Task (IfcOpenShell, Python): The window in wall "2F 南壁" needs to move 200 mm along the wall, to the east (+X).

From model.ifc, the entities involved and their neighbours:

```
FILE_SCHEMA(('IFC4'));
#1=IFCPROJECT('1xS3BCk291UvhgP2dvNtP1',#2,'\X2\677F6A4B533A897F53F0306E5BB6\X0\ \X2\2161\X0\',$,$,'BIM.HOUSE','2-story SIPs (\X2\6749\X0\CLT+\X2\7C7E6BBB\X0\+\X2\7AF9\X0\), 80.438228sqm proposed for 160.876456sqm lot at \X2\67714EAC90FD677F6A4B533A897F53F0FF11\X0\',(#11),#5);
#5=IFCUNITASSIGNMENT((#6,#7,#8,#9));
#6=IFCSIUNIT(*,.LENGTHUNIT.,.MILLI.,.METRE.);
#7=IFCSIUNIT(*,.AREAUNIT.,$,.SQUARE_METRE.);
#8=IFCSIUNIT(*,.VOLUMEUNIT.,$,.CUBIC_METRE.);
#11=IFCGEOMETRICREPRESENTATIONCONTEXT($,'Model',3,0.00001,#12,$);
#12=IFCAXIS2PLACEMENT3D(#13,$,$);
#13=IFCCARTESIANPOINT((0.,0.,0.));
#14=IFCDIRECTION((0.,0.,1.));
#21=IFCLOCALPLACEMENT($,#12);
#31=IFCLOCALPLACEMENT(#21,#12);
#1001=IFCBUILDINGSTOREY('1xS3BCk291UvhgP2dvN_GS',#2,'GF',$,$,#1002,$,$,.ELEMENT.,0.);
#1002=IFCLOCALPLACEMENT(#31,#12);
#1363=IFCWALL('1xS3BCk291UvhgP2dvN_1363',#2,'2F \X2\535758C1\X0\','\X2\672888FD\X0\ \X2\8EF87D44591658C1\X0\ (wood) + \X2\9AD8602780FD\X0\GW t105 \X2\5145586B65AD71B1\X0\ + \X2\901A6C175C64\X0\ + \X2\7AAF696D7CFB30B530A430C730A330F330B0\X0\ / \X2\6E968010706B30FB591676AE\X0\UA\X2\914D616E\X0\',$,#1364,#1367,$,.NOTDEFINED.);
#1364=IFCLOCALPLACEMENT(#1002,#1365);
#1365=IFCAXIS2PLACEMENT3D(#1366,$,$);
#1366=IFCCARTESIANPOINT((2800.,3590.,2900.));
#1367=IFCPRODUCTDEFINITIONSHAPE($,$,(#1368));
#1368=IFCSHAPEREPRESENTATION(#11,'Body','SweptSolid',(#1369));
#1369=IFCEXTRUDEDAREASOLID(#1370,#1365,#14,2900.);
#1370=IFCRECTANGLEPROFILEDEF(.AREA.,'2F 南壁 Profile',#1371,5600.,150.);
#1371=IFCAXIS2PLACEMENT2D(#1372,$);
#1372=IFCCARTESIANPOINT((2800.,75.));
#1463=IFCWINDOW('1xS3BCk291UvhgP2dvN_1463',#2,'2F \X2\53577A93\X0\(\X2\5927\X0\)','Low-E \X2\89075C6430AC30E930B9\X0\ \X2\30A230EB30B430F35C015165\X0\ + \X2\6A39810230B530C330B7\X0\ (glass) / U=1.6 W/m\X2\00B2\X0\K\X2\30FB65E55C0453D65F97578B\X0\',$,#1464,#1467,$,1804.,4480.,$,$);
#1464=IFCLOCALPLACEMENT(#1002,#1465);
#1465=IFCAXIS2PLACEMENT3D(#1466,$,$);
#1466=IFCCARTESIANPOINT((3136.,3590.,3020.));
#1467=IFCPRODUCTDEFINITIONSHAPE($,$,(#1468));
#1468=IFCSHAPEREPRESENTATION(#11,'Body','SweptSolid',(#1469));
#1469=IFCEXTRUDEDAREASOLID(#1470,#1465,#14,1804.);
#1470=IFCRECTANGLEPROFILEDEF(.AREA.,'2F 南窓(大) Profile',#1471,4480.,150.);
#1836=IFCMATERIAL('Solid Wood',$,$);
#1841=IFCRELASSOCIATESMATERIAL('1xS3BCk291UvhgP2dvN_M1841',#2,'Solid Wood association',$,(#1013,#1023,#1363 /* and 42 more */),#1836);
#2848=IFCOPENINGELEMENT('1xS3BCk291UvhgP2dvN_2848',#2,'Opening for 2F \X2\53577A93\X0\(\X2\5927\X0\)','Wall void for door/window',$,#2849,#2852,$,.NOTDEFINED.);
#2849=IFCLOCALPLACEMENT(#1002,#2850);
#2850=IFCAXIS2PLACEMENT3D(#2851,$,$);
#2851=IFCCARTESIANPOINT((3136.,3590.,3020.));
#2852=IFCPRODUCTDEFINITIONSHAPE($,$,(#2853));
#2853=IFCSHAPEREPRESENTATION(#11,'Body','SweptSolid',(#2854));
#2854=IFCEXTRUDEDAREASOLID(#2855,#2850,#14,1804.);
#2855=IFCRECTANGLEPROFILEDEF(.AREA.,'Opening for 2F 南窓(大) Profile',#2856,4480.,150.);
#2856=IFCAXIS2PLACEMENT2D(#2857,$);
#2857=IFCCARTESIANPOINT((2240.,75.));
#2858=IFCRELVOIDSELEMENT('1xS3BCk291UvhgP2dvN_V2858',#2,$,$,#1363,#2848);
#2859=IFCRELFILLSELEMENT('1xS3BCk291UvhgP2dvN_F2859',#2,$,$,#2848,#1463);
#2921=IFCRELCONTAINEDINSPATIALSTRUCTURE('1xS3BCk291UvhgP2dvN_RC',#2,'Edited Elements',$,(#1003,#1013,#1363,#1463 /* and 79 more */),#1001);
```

```python
import ifcopenshell
import ifcopenshell.api.geometry
import ifcopenshell.util.placement
import ifcopenshell.util.unit

model = ifcopenshell.open("model.ifc")
unit_scale = ifcopenshell.util.unit.calculate_unit_scale(model)

window = model.by_id(1463)
opening = window.FillsVoids[0].RelatingOpeningElement
wall = opening.VoidsElements[0].RelatingBuildingElement

wall_matrix = ifcopenshell.util.placement.get_local_placement(wall.ObjectPlacement)
shift = wall_matrix[:3, 0] * 0.2 / unit_scale
before = ifcopenshell.util.placement.get_local_placement(window.ObjectPlacement)[:3, 3].copy()

# The window is not placed relative to its opening, so move both.
for product in (opening, window):
    matrix = ifcopenshell.util.placement.get_local_placement(product.ObjectPlacement)
    matrix[:3, 3] += shift
    ifcopenshell.api.geometry.edit_object_placement(model, product=product, matrix=matrix, is_si=False)

after = ifcopenshell.util.placement.get_local_placement(window.ObjectPlacement)[:3, 3]
print("window moved by", (after - before).round(3) + 0.0)

model.write("model-out.ifc")
```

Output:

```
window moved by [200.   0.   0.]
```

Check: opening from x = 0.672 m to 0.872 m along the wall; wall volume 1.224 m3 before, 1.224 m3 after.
